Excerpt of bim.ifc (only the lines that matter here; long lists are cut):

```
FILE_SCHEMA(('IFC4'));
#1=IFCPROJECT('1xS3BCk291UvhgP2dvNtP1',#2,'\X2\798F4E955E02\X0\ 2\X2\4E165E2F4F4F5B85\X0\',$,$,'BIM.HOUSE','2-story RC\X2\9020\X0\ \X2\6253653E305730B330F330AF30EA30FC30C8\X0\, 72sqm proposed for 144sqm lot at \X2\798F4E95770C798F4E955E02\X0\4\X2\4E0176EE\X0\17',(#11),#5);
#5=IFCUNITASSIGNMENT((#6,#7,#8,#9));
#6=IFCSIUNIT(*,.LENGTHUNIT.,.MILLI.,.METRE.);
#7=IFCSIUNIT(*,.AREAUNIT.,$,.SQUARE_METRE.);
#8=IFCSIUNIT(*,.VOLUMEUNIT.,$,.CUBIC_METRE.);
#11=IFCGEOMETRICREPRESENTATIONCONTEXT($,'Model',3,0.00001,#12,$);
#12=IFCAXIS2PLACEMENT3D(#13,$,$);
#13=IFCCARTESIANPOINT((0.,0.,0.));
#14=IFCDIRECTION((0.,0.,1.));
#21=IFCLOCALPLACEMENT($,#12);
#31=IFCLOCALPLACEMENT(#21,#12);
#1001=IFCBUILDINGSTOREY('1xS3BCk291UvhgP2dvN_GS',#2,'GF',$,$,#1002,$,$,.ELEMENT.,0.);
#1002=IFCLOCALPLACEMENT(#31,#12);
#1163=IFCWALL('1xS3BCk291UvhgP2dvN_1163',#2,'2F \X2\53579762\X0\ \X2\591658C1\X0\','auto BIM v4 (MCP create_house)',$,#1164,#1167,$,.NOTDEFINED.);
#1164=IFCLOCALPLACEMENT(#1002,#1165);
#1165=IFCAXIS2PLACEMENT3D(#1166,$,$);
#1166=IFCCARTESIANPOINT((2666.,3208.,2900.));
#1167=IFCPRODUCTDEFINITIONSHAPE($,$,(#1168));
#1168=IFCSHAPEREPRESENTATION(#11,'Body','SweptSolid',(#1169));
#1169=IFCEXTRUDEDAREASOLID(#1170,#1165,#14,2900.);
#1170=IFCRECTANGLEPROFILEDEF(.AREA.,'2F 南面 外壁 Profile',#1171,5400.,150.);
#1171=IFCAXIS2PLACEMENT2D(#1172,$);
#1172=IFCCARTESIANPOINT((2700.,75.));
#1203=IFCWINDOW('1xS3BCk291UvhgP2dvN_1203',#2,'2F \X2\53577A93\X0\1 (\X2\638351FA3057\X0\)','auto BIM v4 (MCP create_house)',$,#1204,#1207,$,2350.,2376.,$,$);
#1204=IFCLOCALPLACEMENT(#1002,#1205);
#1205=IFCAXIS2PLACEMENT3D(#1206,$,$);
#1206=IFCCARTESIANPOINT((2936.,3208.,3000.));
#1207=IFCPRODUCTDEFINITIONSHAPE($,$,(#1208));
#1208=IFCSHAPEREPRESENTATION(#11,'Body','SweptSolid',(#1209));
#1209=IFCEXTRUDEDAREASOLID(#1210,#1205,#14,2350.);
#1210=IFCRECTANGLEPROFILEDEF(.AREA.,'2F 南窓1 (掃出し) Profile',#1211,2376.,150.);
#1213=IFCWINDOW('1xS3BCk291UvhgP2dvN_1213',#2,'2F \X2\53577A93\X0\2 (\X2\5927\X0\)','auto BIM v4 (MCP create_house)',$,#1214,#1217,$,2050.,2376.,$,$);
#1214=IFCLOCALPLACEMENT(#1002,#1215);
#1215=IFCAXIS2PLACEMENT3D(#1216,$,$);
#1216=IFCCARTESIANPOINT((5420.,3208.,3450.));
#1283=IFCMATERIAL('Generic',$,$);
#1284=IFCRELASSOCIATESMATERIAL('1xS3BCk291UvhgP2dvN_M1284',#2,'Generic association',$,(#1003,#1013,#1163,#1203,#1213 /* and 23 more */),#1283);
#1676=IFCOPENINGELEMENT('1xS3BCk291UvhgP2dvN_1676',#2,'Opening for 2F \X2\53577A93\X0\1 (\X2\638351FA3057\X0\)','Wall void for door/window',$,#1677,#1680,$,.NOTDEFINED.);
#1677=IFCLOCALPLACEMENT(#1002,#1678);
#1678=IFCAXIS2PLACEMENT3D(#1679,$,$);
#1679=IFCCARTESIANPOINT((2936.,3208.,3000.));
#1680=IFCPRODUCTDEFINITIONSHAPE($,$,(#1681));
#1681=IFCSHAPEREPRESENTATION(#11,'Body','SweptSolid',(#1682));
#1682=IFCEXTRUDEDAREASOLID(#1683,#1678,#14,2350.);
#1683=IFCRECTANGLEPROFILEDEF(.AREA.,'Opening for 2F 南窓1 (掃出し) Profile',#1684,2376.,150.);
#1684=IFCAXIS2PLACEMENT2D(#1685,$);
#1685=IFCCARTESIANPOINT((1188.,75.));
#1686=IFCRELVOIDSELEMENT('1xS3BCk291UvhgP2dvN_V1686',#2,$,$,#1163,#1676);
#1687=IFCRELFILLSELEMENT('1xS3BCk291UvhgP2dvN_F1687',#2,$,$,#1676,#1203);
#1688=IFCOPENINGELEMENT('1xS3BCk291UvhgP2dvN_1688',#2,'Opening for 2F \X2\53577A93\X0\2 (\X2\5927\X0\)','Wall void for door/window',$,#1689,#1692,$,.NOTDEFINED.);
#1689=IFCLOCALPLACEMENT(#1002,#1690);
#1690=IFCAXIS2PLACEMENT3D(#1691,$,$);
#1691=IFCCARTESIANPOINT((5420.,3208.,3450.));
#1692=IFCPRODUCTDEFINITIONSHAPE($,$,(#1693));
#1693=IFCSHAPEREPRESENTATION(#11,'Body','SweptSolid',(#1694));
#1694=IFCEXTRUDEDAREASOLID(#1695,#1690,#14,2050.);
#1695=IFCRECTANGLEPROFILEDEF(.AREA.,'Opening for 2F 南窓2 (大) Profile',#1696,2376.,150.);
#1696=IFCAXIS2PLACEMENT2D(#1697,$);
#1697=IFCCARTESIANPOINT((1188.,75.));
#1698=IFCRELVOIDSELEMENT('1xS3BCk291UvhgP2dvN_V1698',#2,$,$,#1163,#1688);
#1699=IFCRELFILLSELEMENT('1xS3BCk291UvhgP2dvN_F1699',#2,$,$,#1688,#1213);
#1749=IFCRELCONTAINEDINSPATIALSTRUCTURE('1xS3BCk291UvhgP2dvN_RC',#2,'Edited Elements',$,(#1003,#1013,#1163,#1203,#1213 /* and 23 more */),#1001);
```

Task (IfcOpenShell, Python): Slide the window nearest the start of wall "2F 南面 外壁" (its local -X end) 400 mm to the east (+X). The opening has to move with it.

```python
import ifcopenshell
import ifcopenshell.api.geometry
import ifcopenshell.util.placement
import ifcopenshell.util.unit

model = ifcopenshell.open("bim.ifc")
unit_scale = ifcopenshell.util.unit.calculate_unit_scale(model)

window = model.by_id(1203)
opening = window.FillsVoids[0].RelatingOpeningElement
wall = opening.VoidsElements[0].RelatingBuildingElement

wall_matrix = ifcopenshell.util.placement.get_local_placement(wall.ObjectPlacement)
shift = wall_matrix[:3, 0] * 0.4 / unit_scale
before = ifcopenshell.util.placement.get_local_placement(window.ObjectPlacement)[:3, 3].copy()

# The window is not placed relative to its opening, so move both.
for product in (opening, window):
    matrix = ifcopenshell.util.placement.get_local_placement(product.ObjectPlacement)
    matrix[:3, 3] += shift
    ifcopenshell.api.geometry.edit_object_placement(model, product=product, matrix=matrix, is_si=False)

after = ifcopenshell.util.placement.get_local_placement(window.ObjectPlacement)[:3, 3]
print("window moved by", (after - before).round(3) + 0.0)

model.write("bim_rev.ifc")
```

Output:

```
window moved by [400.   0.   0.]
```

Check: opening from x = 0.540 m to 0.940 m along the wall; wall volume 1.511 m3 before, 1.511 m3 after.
